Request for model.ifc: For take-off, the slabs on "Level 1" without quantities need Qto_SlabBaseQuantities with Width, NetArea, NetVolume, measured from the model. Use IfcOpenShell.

First a look at what the model holds.

```python
import ifcopenshell
import ifcopenshell.util.element
import ifcopenshell.util.unit

model = ifcopenshell.open("model.ifc")
print(model.schema)
for unit_type in ("LENGTHUNIT", "AREAUNIT", "VOLUMEUNIT"):
    print(unit_type, ifcopenshell.util.unit.calculate_unit_scale(model, unit_type))
storey = next(s for s in model.by_type("IfcBuildingStorey") if s.Name == "Level 1")
slabs = [e for e in ifcopenshell.util.element.get_decomposition(storey) if e.is_a("IfcSlab")]
for e in sorted(slabs, key=lambda e: e.id()):
    print(e.id(), e.is_a(), e.Name, list(ifcopenshell.util.element.get_psets(e, qtos_only=True)), sep=" | ")
```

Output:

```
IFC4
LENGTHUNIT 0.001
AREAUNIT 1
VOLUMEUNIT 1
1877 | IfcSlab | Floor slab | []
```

```python
import ifcopenshell
import ifcopenshell.api.pset
import ifcopenshell.geom
import ifcopenshell.util.element
import ifcopenshell.util.shape
import ifcopenshell.util.unit

model = ifcopenshell.open("model.ifc")
unit_scale = ifcopenshell.util.unit.calculate_unit_scale(model)
area_scale = ifcopenshell.util.unit.calculate_unit_scale(model, "AREAUNIT")
volume_scale = ifcopenshell.util.unit.calculate_unit_scale(model, "VOLUMEUNIT")
settings = ifcopenshell.geom.settings()

storey = next(s for s in model.by_type("IfcBuildingStorey") if s.Name == "Level 1")
slabs = [e for e in ifcopenshell.util.element.get_decomposition(storey) if e.is_a("IfcSlab")]

for e in sorted(slabs, key=lambda e: e.id()):
    if ifcopenshell.util.element.get_psets(e, qtos_only=True, should_inherit=False):
        continue
    # Geometry comes back in metres, in the element's own axes.
    shape = ifcopenshell.geom.create_shape(settings, e)
    values = {
        "Width": ifcopenshell.util.shape.get_z(shape.geometry) / unit_scale,
        "NetArea": ifcopenshell.util.shape.get_footprint_area(shape.geometry) / area_scale,
        "NetVolume": ifcopenshell.util.shape.get_volume(shape.geometry) / volume_scale,
    }
    qto = ifcopenshell.api.pset.add_qto(model, product=e, name="Qto_SlabBaseQuantities")
    ifcopenshell.api.pset.edit_qto(model, qto=qto, properties=values)
    print(e.id(), {k: round(v, 3) for k, v in values.items()})

model.write("model_v2.ifc")
```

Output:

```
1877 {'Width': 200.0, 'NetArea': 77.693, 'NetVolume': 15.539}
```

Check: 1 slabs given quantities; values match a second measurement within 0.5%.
